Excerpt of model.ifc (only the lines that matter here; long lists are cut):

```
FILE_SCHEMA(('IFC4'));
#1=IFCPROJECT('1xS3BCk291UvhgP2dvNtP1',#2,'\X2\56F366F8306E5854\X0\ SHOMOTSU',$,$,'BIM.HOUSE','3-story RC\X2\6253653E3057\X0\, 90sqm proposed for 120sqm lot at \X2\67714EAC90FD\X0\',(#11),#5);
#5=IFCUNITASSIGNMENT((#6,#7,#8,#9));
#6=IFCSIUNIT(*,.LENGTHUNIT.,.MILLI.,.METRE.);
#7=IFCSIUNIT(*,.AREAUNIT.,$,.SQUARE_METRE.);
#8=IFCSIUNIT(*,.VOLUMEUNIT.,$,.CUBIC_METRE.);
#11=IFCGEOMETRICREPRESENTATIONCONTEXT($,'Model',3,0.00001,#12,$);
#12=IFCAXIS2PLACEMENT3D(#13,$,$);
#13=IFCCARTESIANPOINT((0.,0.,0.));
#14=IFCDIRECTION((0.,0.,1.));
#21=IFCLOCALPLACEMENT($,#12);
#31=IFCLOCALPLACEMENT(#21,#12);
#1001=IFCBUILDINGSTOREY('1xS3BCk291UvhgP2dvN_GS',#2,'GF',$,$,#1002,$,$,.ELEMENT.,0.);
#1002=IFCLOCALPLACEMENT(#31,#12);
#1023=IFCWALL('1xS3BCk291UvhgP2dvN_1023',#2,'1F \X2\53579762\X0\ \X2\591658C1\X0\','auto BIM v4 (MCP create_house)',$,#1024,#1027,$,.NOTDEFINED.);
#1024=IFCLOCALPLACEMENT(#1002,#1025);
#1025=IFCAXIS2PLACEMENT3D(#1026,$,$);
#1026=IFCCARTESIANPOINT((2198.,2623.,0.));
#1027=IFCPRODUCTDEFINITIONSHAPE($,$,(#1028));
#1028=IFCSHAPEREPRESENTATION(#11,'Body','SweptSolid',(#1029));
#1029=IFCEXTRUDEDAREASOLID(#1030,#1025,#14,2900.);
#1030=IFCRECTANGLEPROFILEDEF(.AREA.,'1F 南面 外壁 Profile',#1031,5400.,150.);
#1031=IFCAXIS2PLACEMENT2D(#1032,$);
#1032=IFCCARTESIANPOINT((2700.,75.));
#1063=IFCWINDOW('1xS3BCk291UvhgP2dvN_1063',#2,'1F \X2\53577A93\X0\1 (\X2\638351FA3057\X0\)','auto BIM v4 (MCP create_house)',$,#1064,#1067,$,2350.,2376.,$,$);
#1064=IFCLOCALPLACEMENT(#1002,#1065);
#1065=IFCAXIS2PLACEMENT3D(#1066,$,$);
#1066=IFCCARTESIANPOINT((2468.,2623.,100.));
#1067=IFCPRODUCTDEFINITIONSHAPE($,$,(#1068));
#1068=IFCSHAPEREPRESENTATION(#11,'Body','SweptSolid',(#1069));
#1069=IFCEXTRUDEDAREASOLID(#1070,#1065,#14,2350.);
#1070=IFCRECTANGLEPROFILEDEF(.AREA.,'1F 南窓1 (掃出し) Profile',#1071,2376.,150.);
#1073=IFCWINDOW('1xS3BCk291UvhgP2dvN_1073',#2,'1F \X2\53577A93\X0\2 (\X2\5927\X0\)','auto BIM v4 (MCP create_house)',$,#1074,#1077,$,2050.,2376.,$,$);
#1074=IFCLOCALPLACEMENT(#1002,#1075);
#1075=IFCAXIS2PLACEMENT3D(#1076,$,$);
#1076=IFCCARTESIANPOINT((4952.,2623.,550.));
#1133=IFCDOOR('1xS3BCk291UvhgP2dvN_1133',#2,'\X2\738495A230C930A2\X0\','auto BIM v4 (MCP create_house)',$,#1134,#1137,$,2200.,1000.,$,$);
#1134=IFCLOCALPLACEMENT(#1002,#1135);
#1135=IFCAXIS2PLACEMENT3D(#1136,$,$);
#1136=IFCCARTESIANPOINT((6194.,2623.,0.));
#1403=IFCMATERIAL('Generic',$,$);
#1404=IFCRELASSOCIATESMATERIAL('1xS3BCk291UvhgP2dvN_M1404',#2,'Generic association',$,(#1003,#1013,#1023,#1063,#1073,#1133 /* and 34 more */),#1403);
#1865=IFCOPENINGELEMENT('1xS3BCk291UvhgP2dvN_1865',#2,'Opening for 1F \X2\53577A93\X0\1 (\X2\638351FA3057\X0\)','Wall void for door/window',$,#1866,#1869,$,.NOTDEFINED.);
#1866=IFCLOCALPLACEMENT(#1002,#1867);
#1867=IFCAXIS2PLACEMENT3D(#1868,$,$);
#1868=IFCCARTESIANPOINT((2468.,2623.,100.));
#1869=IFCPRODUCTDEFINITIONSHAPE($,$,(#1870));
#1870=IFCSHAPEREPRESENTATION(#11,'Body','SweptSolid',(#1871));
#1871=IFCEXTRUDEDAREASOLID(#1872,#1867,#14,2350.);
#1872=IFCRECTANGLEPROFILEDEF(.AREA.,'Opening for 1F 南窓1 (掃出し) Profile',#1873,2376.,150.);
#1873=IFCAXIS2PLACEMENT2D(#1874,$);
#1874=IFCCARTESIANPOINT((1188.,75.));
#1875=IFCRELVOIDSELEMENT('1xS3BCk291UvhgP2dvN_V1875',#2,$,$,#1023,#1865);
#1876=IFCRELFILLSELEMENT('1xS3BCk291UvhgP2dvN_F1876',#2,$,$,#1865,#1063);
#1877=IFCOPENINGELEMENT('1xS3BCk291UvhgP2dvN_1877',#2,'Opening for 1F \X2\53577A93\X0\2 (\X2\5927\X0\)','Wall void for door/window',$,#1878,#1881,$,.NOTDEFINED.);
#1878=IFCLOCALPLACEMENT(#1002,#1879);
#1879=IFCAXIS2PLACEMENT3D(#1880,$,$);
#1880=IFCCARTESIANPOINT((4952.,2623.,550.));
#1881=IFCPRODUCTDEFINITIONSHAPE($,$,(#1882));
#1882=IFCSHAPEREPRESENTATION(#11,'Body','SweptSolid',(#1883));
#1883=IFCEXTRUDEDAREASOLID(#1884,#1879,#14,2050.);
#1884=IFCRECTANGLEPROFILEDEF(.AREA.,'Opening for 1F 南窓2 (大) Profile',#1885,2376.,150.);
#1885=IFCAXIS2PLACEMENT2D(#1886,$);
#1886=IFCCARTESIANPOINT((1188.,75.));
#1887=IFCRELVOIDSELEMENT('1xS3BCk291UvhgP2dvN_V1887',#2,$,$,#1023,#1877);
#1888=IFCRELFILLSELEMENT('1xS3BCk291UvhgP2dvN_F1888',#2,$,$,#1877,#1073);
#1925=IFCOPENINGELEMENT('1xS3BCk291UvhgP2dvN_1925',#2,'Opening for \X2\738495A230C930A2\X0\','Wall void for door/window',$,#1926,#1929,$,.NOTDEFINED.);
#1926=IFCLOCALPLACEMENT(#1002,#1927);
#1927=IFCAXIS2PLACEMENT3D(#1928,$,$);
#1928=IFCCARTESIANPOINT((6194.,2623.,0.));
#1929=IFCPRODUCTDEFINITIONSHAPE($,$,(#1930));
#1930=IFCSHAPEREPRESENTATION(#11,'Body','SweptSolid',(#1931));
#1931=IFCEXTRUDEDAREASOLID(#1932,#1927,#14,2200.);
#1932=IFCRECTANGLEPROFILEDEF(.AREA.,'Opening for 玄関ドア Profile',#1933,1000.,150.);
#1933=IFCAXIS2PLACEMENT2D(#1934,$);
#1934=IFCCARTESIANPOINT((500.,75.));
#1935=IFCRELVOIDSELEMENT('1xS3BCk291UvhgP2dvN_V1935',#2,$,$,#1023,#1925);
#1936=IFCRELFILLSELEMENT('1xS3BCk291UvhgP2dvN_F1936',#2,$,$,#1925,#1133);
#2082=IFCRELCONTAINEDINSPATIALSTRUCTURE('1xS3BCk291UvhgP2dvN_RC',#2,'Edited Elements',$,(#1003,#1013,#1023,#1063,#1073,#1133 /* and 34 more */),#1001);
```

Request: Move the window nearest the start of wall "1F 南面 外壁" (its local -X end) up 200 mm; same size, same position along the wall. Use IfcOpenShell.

```python
import numpy as np
import ifcopenshell
import ifcopenshell.api.geometry
import ifcopenshell.util.placement
import ifcopenshell.util.unit

model = ifcopenshell.open("model.ifc")
unit_scale = ifcopenshell.util.unit.calculate_unit_scale(model)

window = model.by_guid("1xS3BCk291UvhgP2dvN_1063")
opening = window.FillsVoids[0].RelatingOpeningElement
dz = 200.0

shift = np.array([0.0, 0.0, dz])
# The window is not placed relative to its opening, so move both.
for product in (opening, window):
    matrix = ifcopenshell.util.placement.get_local_placement(product.ObjectPlacement)
    matrix[:3, 3] += shift
    ifcopenshell.api.geometry.edit_object_placement(model, product=product, matrix=matrix, is_si=False)

print(f"moved by {dz * unit_scale:+.3f} m")

model.write("model-out.ifc")
```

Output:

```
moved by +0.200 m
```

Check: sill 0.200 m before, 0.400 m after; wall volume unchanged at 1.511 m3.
